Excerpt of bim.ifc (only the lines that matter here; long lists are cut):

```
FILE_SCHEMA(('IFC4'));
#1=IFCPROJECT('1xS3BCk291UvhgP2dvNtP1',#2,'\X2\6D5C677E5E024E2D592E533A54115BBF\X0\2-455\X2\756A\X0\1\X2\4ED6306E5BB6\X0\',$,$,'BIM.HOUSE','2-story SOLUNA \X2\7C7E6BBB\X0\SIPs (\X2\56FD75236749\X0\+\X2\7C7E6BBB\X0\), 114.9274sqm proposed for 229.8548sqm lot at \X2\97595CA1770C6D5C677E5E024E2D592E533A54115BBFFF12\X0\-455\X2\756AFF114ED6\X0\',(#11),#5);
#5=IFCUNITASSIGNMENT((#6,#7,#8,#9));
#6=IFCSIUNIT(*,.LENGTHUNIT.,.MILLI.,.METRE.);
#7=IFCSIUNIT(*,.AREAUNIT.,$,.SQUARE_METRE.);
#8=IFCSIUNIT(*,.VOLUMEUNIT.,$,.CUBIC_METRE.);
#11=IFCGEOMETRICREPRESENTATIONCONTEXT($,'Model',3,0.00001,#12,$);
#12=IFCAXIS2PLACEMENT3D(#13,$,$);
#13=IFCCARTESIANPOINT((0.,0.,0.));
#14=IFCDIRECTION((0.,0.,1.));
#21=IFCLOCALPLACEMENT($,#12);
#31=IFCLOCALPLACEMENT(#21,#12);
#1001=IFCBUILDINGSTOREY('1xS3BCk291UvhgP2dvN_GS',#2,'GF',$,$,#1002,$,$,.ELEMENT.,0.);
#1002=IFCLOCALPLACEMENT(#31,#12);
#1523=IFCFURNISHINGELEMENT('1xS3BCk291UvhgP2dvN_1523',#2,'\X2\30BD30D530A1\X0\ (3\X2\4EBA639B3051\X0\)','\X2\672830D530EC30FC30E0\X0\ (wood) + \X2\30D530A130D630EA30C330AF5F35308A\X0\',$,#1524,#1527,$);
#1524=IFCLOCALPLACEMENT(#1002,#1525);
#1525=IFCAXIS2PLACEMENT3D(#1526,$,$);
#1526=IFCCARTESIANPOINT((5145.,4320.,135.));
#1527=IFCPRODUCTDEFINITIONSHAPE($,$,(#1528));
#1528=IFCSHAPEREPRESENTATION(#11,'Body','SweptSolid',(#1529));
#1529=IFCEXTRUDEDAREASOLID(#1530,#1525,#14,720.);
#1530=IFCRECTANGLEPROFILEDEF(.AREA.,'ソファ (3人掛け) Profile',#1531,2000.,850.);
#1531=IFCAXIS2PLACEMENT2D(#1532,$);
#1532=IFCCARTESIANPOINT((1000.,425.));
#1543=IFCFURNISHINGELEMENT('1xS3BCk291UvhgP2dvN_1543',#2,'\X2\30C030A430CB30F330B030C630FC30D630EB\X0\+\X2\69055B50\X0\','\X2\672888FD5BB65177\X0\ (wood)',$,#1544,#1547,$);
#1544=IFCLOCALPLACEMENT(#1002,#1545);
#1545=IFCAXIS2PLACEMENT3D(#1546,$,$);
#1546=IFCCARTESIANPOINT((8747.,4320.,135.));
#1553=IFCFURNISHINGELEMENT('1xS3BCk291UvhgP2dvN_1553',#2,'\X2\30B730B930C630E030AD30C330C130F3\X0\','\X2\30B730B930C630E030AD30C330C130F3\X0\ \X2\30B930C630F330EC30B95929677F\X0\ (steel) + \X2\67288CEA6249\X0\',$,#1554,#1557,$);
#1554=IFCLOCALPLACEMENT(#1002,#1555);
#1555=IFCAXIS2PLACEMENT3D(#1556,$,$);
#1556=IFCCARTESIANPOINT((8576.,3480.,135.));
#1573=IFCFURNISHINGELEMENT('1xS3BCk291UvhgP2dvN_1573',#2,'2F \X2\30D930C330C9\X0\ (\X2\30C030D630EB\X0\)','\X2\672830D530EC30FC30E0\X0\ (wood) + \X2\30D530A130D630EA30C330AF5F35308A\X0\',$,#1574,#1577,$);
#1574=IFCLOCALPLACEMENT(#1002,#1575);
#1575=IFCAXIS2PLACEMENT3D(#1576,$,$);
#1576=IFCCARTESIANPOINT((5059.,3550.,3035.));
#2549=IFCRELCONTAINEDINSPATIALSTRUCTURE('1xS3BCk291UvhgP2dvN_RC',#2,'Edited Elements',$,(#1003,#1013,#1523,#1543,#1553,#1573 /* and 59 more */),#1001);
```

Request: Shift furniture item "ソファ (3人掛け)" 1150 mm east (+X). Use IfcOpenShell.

```python
import ifcopenshell
import ifcopenshell.api.geometry
import ifcopenshell.util.placement
import ifcopenshell.util.unit

model = ifcopenshell.open("bim.ifc")
unit_scale = ifcopenshell.util.unit.calculate_unit_scale(model)

item = model.by_guid("1xS3BCk291UvhgP2dvN_1523")
matrix = ifcopenshell.util.placement.get_local_placement(item.ObjectPlacement)
matrix[0, 3] += 1.15 / unit_scale
ifcopenshell.api.geometry.edit_object_placement(model, product=item, matrix=matrix, is_si=False)

print(ifcopenshell.util.placement.get_local_placement(item.ObjectPlacement).round(3) + 0.0)

model.write("bim_updated.ifc")
```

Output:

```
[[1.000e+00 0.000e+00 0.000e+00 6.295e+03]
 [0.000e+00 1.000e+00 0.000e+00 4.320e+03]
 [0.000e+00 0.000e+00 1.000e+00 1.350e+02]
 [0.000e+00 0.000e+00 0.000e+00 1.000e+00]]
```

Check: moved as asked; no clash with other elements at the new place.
